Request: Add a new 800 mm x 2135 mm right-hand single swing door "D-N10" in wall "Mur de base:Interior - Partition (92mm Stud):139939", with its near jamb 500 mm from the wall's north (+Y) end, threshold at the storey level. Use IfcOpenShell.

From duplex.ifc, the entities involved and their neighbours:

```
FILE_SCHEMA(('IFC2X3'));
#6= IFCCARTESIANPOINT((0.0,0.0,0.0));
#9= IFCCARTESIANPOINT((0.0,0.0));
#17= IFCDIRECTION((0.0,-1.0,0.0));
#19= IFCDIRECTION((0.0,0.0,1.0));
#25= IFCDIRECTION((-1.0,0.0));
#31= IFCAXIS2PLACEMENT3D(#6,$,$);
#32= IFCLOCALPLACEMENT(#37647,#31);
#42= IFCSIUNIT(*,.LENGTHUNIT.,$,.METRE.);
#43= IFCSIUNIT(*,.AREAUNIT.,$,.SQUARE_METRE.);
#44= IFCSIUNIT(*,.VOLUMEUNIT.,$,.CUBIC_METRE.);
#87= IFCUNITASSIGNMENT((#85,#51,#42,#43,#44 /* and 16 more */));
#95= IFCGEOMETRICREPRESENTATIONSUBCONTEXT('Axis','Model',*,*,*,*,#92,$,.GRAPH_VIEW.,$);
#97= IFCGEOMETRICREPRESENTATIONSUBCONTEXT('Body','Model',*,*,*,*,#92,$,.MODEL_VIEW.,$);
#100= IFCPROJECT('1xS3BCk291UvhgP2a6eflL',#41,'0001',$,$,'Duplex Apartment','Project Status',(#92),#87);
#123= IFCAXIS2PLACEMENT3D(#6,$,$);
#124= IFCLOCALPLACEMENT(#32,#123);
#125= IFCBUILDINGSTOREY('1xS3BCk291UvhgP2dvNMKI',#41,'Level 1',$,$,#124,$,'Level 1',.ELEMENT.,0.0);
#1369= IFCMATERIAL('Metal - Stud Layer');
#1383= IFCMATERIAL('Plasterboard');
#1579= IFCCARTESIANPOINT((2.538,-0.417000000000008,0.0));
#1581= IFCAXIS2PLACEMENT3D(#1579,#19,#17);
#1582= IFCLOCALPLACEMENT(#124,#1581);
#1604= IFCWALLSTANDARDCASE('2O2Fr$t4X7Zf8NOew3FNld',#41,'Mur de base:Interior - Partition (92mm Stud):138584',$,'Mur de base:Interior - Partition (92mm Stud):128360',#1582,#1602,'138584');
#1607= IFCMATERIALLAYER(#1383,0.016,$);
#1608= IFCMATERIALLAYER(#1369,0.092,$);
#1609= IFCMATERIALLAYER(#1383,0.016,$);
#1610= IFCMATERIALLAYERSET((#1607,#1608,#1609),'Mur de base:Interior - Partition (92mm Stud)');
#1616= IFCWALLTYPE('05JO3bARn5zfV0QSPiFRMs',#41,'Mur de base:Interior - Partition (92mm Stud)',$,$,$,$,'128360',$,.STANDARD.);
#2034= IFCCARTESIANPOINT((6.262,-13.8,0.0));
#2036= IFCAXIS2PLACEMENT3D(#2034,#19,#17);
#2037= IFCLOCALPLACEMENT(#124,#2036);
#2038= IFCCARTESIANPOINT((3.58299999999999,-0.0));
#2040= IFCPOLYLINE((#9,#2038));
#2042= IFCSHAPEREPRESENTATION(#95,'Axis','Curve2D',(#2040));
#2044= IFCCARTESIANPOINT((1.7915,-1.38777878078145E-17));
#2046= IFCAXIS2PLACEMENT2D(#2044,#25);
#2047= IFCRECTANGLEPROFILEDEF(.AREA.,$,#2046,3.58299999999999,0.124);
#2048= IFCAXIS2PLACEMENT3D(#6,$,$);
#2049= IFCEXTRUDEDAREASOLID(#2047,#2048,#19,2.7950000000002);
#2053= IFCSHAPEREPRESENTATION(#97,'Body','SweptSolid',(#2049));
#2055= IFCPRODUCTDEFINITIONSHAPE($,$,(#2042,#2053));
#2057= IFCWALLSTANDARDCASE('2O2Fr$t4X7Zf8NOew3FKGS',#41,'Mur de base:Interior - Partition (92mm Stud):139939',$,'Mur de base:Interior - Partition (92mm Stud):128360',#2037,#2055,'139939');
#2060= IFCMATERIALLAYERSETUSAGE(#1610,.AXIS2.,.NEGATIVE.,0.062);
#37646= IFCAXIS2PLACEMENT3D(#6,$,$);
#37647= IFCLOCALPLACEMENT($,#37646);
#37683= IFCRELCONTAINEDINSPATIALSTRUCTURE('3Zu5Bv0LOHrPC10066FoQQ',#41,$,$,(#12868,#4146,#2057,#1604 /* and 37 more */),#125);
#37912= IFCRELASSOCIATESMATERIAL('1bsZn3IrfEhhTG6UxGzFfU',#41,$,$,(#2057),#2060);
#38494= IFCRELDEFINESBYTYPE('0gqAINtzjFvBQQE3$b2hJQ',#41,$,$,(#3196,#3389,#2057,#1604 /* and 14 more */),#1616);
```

```python
import numpy as np
import ifcopenshell
import ifcopenshell.api.feature
import ifcopenshell.api.geometry
import ifcopenshell.api.root
import ifcopenshell.api.spatial
import ifcopenshell.api.type
import ifcopenshell.geom
import ifcopenshell.util.element
import ifcopenshell.util.placement
import ifcopenshell.util.representation
import ifcopenshell.util.shape
import ifcopenshell.util.unit

model = ifcopenshell.open("duplex.ifc")
unit_scale = ifcopenshell.util.unit.calculate_unit_scale(model)
settings = ifcopenshell.geom.settings()


def volume(element):
    """Net volume in cubic metres, openings subtracted."""
    shape = ifcopenshell.geom.create_shape(settings, element)
    return ifcopenshell.util.shape.get_volume(shape.geometry)


wall = model.by_guid("2O2Fr$t4X7Zf8NOew3FKGS")
storey = ifcopenshell.util.element.get_container(wall, ifc_class="IfcBuildingStorey")
context = ifcopenshell.util.representation.get_context(model, "Model", "Body", "MODEL_VIEW")
before = volume(wall)

width, height, from_end, sill = 0.8, 2.135, 0.5, 0.0  # metres

# The wall runs along its own X axis, and the end named is its -X end.
wall_shape = ifcopenshell.geom.create_shape(settings, wall)
x, y, z = ifcopenshell.util.shape.get_vertices(wall_shape.geometry).T
start = x.min() + from_end
face, thickness = float(y.min()), float(y.max() - y.min())
wall_matrix = ifcopenshell.util.placement.get_local_placement(wall.ObjectPlacement)
level = ifcopenshell.util.placement.get_local_placement(storey.ObjectPlacement)[2, 3]


def in_wall(x, y):
    """Placement at x, y metres in the wall's axes, at sill height."""
    matrix = wall_matrix.copy()
    matrix[:, 3] = wall_matrix @ np.array([x / unit_scale, y / unit_scale, 0.0, 1.0])
    matrix[2, 3] = level + sill / unit_scale
    return matrix


# Opening: a box that overshoots both wall faces by 50 mm.
opening = ifcopenshell.api.root.create_entity(model, ifc_class="IfcOpeningElement")
box = ifcopenshell.api.geometry.add_wall_representation(
    model, context=context, length=width, height=height, thickness=thickness + 0.1
)
ifcopenshell.api.geometry.assign_representation(model, product=opening, representation=box)
ifcopenshell.api.geometry.edit_object_placement(model, product=opening, matrix=in_wall(start, face - 0.05), is_si=False)
ifcopenshell.api.feature.add_feature(model, feature=opening, element=wall)

door = ifcopenshell.api.root.create_entity(model, ifc_class="IfcDoor", name="D-N10")
door.OverallWidth, door.OverallHeight = width / unit_scale, height / unit_scale
body = ifcopenshell.api.geometry.add_door_representation(
    model,
    context=context,
    overall_width=door.OverallWidth,
    overall_height=door.OverallHeight,
    operation_type="SINGLE_SWING_RIGHT",
    lining_properties={"LiningDepth": thickness / unit_scale, "ThresholdDepth": thickness / unit_scale},
)
ifcopenshell.api.geometry.assign_representation(model, product=door, representation=body)
ifcopenshell.api.spatial.assign_container(model, products=[door], relating_structure=storey)
fills = ifcopenshell.api.feature.add_filling(model, opening=opening, element=door)
fills.OwnerHistory = door.OwnerHistory  # required in IFC2X3

# IFC2X3 keeps the operation on the door style.
style = ifcopenshell.api.root.create_entity(model, ifc_class="IfcDoorStyle", name="D-N10")
style.OperationType, style.ConstructionType = "SINGLE_SWING_RIGHT", "NOTDEFINED"
style.ParameterTakesPrecedence = style.Sizeable = False
ifcopenshell.api.type.assign_type(model, related_objects=[door], relating_type=style)

# The lining spans the wall, so the door starts at the wall face.
ifcopenshell.api.geometry.edit_object_placement(model, product=door, matrix=in_wall(start, face), is_si=False)

after = volume(wall)

print(f"wall volume {before:.3f} -> {after:.3f} m3")

model.write("duplex_edited.ifc")
```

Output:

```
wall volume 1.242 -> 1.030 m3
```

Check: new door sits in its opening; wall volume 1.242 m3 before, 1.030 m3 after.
